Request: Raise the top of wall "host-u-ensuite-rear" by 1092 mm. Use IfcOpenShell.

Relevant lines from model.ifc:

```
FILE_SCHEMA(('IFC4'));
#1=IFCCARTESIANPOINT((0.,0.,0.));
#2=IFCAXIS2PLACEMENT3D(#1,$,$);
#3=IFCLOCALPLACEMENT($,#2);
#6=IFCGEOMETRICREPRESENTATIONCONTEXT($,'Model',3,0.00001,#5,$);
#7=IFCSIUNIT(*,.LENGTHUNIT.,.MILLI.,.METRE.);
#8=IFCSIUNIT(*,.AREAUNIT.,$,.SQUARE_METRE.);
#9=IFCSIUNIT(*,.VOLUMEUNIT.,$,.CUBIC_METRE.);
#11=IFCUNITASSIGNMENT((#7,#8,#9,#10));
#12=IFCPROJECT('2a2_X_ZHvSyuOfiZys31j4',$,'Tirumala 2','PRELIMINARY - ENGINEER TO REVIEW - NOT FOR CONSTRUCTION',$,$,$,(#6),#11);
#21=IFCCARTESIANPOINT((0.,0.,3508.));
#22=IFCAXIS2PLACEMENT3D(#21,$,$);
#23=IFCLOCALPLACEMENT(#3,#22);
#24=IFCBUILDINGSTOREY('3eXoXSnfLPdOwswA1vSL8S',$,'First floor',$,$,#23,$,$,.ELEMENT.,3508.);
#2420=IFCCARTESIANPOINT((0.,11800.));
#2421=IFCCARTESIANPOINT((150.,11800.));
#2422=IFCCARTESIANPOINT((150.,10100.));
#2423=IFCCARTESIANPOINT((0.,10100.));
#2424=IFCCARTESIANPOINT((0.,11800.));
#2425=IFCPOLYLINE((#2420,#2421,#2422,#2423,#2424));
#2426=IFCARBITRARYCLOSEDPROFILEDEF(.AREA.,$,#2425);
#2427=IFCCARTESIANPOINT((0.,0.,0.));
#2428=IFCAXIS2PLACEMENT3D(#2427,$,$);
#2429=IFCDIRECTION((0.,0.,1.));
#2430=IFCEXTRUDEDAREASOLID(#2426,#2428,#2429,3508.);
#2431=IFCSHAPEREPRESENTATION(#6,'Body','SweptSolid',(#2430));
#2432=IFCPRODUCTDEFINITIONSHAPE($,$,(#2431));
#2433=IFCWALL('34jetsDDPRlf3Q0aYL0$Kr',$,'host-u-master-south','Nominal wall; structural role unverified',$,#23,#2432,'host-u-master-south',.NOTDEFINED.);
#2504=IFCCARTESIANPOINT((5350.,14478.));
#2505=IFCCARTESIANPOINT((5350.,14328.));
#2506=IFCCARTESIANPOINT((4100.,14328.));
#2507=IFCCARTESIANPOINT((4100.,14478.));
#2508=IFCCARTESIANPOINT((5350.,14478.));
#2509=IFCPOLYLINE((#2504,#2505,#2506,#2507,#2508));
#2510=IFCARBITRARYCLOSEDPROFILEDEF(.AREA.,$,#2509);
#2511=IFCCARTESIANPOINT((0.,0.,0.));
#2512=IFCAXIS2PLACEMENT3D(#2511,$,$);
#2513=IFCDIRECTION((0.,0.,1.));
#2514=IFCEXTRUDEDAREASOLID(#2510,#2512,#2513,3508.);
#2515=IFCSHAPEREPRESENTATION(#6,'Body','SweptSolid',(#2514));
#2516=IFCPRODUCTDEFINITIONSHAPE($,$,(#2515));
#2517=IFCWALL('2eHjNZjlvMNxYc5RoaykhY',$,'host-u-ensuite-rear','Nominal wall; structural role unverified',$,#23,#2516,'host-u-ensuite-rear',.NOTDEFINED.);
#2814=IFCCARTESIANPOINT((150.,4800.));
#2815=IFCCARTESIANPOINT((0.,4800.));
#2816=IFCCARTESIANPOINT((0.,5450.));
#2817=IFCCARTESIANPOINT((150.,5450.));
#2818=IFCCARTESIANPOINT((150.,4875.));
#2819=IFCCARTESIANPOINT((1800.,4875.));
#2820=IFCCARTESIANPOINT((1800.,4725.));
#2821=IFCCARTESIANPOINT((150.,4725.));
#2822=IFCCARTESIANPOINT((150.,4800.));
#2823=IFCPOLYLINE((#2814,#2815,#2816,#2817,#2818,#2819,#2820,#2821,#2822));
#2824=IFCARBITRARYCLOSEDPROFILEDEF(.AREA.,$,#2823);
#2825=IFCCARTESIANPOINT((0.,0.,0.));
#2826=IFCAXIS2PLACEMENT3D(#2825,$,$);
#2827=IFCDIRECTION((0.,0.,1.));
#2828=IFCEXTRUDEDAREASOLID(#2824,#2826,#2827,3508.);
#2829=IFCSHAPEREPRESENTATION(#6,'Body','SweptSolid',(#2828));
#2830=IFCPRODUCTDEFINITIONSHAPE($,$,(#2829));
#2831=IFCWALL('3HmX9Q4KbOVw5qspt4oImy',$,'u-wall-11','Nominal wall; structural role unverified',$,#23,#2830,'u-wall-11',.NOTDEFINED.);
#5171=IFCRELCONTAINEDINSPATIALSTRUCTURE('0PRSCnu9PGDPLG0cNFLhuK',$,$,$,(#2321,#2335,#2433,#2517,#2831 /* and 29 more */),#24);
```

```python
import ifcopenshell
import ifcopenshell.geom
import ifcopenshell.util.shape

model = ifcopenshell.open("model.ifc")
settings = ifcopenshell.geom.settings()


def volume(element):
    """Net volume in cubic metres, openings subtracted."""
    shape = ifcopenshell.geom.create_shape(settings, element)
    return ifcopenshell.util.shape.get_volume(shape.geometry)


wall = model.by_guid("2eHjNZjlvMNxYc5RoaykhY")
before = volume(wall)

body = next(r for r in wall.Representation.Representations if r.RepresentationIdentifier == "Body")
solid = body.Items[0]
old_height = solid.Depth
solid.Depth += 1092.0
after = volume(wall)

print(f"height {old_height:g} -> {solid.Depth:g}, volume {before:.3f} -> {after:.3f} m3")

model.write("model_updated.ifc")
```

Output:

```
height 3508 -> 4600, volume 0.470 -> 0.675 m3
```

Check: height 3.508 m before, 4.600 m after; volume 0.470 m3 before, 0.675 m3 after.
